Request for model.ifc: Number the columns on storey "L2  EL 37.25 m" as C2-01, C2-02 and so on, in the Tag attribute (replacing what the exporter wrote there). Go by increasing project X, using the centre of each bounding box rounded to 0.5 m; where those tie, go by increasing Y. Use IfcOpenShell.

First a look at what the model holds.

```python
import ifcopenshell
import ifcopenshell.util.element
import ifcopenshell.util.placement

model = ifcopenshell.open("model.ifc")
print(model.schema)
storey = next(s for s in model.by_type("IfcBuildingStorey") if s.Name == "L2  EL 37.25 m")
columns = [e for e in ifcopenshell.util.element.get_decomposition(storey) if e.is_a("IfcColumn")]
for e in sorted(columns, key=lambda e: e.id()):
    origin = ifcopenshell.util.placement.get_local_placement(e.ObjectPlacement)[:3, 3]
    print(e.id(), e.Tag, e.Name, origin.round(2) + 0.0, sep=" | ")
```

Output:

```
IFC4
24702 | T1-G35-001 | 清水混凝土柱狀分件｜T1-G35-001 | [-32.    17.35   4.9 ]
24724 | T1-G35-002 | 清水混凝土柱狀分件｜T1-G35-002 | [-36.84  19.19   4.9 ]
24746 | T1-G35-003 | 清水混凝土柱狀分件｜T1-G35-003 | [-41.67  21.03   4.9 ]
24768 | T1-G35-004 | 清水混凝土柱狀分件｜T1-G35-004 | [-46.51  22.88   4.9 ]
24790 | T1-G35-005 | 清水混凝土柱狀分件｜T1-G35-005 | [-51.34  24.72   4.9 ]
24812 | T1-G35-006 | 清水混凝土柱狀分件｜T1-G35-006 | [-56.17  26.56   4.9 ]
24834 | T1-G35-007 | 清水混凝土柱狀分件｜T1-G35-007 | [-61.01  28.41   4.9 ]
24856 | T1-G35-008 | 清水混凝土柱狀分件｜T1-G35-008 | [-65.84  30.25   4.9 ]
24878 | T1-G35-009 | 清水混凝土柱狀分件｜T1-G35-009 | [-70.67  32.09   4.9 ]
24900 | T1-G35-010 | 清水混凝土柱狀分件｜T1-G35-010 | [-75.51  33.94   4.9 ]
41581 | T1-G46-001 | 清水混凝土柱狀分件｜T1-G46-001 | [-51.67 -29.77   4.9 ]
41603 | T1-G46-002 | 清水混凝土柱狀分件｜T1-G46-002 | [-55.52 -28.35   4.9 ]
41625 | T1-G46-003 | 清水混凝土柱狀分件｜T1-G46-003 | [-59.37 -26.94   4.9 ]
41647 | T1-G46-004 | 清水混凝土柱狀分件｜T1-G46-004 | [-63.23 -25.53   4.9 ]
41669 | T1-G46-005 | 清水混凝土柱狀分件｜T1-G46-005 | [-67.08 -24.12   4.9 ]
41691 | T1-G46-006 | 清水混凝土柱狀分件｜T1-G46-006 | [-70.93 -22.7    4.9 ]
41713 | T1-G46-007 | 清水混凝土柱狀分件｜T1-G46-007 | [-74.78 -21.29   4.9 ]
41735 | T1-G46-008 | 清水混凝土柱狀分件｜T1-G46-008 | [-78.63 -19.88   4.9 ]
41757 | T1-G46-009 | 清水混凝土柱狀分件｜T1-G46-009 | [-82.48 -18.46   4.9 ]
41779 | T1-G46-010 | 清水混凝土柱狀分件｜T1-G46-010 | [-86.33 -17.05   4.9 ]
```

```python
import ifcopenshell
import ifcopenshell.geom
import ifcopenshell.util.element
import ifcopenshell.util.shape

model = ifcopenshell.open("model.ifc")
settings = ifcopenshell.geom.settings()
settings.set("use-world-coords", True)


def centre(element):
    shape = ifcopenshell.geom.create_shape(settings, element)
    return ifcopenshell.util.shape.get_bbox_centroid(shape.geometry)


storey = next(s for s in model.by_type("IfcBuildingStorey") if s.Name == "L2  EL 37.25 m")
columns = [e for e in ifcopenshell.util.element.get_decomposition(storey) if e.is_a("IfcColumn")]

# Insertion points can sit at a corner or the storey origin, so sort by the geometry (in metres).
centres = {e: centre(e) for e in columns}
columns.sort(key=lambda e: (round(centres[e][0] / 0.5), centres[e][1]))

for i, e in enumerate(columns, start=1):
    number = f"C2-{i:02d}"
    e.Tag = number
    print(e.id(), number)

model.write("model-out.ifc")
```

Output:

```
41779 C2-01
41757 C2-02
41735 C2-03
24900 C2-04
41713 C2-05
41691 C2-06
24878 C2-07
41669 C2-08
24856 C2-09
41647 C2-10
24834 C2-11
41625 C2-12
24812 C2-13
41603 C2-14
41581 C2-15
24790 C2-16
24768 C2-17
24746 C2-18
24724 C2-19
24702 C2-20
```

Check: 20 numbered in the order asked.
